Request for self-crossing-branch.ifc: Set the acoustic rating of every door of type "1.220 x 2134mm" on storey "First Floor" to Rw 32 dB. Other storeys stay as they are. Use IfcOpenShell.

First a look at what the model holds.

```python
import ifcopenshell
import ifcopenshell.util.element

model = ifcopenshell.open("self-crossing-branch.ifc")
print(model.schema)
storey = next(s for s in model.by_type("IfcBuildingStorey") if s.Name == "First Floor")
doors = [e for e in ifcopenshell.util.element.get_decomposition(storey) if e.is_a("IfcDoor")]
seen = {}
for e in doors:
    element_type = ifcopenshell.util.element.get_type(e)
    key = (element_type.Name if element_type != e and element_type else None, ifcopenshell.util.element.get_pset(e, "Pset_DoorCommon", "AcousticRating"))
    seen[key] = seen.get(key, 0) + 1
for (name, value), count in sorted(seen.items(), key=str):
    print(count, "x", name, "|", value)
```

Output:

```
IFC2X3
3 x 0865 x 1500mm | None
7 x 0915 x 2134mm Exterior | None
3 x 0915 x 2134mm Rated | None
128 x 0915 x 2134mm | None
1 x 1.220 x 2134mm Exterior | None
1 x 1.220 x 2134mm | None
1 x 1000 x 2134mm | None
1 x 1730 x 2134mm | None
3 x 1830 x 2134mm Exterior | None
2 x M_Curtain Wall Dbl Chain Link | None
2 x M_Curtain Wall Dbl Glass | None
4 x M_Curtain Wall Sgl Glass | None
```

```python
import ifcopenshell
import ifcopenshell.api.pset
import ifcopenshell.util.element

model = ifcopenshell.open("self-crossing-branch.ifc")

storey = next(s for s in model.by_type("IfcBuildingStorey") if s.Name == "First Floor")
doors = [e for e in ifcopenshell.util.element.get_decomposition(storey) if e.is_a("IfcDoor")]

count = 0
for e in doors:
    element_type = ifcopenshell.util.element.get_type(e)
    if element_type in (None, e) or element_type.Name != "1.220 x 2134mm":
        continue
    # add_pset returns the element's existing set when there is one.
    pset = ifcopenshell.api.pset.add_pset(model, product=e, name="Pset_DoorCommon")
    ifcopenshell.api.pset.edit_pset(model, pset=pset, properties={"AcousticRating": "Rw 32 dB"})
    count += 1

print(count, "doors updated")

model.write("self-crossing-branch_v2.ifc")
```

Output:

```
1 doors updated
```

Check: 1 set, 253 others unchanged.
